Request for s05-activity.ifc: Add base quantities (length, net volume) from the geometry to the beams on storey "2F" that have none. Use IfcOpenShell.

First a look at what the model holds.

```python
import ifcopenshell
import ifcopenshell.util.element
import ifcopenshell.util.unit

model = ifcopenshell.open("s05-activity.ifc")
print(model.schema)
for unit_type in ("LENGTHUNIT", "AREAUNIT", "VOLUMEUNIT"):
    print(unit_type, ifcopenshell.util.unit.calculate_unit_scale(model, unit_type))
storey = next(s for s in model.by_type("IfcBuildingStorey") if s.Name == "2F")
beams = [e for e in ifcopenshell.util.element.get_decomposition(storey) if e.is_a("IfcBeam")]
for e in sorted(beams, key=lambda e: e.id()):
    print(e.id(), e.is_a(), e.Name, list(ifcopenshell.util.element.get_psets(e, qtos_only=True)), sep=" | ")
```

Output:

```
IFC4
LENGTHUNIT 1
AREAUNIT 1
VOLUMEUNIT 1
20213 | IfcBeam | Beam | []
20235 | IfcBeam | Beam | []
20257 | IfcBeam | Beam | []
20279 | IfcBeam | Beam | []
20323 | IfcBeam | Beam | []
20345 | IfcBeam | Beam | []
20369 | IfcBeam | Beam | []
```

```python
import ifcopenshell
import ifcopenshell.api.pset
import ifcopenshell.geom
import ifcopenshell.util.element
import ifcopenshell.util.shape
import ifcopenshell.util.unit

model = ifcopenshell.open("s05-activity.ifc")
unit_scale = ifcopenshell.util.unit.calculate_unit_scale(model)
volume_scale = ifcopenshell.util.unit.calculate_unit_scale(model, "VOLUMEUNIT")
settings = ifcopenshell.geom.settings()

storey = next(s for s in model.by_type("IfcBuildingStorey") if s.Name == "2F")
beams = [e for e in ifcopenshell.util.element.get_decomposition(storey) if e.is_a("IfcBeam")]

for e in sorted(beams, key=lambda e: e.id()):
    if ifcopenshell.util.element.get_psets(e, qtos_only=True, should_inherit=False):
        continue
    # Geometry comes back in metres, in the element's own axes.
    shape = ifcopenshell.geom.create_shape(settings, e)
    values = {
        "Length": ifcopenshell.util.shape.get_max_xyz(shape.geometry) / unit_scale,
        "NetVolume": ifcopenshell.util.shape.get_volume(shape.geometry) / volume_scale,
    }
    qto = ifcopenshell.api.pset.add_qto(model, product=e, name="Qto_BeamBaseQuantities")
    ifcopenshell.api.pset.edit_qto(model, qto=qto, properties=values)
    print(e.id(), {k: round(v, 3) for k, v in values.items()})

model.write("s05-activity-out.ifc")
```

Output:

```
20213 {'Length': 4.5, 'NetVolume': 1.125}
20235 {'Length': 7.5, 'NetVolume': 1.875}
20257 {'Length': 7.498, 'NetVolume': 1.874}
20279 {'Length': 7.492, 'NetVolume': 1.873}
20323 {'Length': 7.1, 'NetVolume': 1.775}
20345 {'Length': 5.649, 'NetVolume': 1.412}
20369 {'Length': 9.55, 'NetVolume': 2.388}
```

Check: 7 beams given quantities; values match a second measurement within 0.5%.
